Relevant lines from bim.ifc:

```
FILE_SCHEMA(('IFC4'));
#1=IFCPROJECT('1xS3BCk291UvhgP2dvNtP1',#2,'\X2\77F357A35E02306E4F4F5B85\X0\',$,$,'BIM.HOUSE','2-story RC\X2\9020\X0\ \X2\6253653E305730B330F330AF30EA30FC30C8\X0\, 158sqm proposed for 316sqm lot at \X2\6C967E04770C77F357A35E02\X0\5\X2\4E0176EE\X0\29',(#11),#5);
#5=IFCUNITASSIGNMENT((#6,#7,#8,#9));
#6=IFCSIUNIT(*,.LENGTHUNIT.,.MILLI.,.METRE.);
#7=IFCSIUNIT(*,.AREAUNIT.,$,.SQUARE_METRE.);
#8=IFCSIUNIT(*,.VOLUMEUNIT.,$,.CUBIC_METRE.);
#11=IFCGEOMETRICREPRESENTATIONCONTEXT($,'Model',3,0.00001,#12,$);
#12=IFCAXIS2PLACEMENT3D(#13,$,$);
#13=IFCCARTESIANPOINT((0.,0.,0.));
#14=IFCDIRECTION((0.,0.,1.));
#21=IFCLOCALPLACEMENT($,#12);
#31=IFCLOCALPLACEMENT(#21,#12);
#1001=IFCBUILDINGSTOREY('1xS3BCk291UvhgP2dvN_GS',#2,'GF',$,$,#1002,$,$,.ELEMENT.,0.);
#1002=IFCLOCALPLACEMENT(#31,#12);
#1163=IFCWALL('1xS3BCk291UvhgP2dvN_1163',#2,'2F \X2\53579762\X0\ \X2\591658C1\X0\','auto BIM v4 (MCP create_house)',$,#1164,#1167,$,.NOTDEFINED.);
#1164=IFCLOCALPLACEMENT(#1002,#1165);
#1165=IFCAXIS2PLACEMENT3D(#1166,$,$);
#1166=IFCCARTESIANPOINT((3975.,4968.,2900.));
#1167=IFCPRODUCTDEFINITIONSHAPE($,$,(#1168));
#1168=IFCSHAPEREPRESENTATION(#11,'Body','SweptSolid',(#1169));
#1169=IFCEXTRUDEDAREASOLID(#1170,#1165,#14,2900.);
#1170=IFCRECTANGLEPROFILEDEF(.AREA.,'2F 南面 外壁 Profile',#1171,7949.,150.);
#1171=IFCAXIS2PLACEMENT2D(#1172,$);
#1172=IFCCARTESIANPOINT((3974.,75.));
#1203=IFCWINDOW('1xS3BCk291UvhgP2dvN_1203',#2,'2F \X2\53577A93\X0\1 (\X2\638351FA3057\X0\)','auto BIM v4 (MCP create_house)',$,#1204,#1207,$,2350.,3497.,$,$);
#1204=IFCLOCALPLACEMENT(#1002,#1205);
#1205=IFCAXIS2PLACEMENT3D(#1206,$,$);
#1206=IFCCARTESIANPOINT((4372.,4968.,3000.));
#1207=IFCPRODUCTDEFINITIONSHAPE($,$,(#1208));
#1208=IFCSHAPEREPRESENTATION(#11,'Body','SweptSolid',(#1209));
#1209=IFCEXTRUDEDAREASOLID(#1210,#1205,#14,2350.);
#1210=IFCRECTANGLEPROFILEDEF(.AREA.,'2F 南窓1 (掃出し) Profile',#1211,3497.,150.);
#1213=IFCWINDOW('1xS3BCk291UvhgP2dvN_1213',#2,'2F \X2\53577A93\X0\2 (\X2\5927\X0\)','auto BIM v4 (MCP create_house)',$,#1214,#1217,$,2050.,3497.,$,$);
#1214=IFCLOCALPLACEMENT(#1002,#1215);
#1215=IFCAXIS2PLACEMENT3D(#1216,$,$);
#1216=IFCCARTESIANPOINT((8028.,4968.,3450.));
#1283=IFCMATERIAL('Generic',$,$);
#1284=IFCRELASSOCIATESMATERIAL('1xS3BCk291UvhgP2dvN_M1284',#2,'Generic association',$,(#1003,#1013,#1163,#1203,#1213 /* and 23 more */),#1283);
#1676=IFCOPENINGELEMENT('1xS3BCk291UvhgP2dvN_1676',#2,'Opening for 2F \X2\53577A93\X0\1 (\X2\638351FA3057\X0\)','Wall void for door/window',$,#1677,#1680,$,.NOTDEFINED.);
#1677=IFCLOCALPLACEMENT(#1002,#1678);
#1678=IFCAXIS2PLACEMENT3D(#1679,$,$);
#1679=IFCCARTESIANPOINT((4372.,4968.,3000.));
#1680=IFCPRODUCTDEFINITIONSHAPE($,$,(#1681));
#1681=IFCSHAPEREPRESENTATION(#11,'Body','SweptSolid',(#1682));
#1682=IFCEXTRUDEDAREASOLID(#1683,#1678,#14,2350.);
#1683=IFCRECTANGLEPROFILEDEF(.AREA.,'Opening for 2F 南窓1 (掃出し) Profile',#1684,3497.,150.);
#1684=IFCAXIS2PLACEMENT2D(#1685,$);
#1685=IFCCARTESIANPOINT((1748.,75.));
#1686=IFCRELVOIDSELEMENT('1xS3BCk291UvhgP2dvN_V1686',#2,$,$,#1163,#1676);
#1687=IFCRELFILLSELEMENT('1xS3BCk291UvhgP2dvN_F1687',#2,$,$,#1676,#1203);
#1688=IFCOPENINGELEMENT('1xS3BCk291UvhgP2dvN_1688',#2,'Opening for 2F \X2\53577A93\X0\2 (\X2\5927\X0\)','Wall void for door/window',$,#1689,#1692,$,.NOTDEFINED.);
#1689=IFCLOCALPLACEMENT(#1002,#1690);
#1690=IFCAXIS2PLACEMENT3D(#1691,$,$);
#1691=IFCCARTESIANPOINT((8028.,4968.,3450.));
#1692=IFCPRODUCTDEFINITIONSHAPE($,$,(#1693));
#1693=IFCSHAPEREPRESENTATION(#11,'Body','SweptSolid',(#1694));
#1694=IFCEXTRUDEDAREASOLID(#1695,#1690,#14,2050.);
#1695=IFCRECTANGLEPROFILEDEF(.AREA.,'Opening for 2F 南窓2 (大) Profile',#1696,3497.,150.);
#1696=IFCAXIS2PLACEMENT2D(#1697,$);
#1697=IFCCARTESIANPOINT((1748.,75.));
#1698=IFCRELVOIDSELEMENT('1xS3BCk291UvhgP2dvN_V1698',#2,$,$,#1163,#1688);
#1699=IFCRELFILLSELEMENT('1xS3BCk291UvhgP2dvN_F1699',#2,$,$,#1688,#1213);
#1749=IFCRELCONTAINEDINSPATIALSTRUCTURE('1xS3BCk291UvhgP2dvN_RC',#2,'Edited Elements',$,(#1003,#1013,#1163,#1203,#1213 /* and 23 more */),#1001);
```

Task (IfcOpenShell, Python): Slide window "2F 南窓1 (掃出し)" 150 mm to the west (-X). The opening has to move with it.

```python
import ifcopenshell
import ifcopenshell.api.geometry
import ifcopenshell.util.placement
import ifcopenshell.util.unit

model = ifcopenshell.open("bim.ifc")
unit_scale = ifcopenshell.util.unit.calculate_unit_scale(model)

window = model.by_guid("1xS3BCk291UvhgP2dvN_1203")
opening = window.FillsVoids[0].RelatingOpeningElement
wall = opening.VoidsElements[0].RelatingBuildingElement

wall_matrix = ifcopenshell.util.placement.get_local_placement(wall.ObjectPlacement)
shift = wall_matrix[:3, 0] * -0.15 / unit_scale
before = ifcopenshell.util.placement.get_local_placement(window.ObjectPlacement)[:3, 3].copy()

# The window is not placed relative to its opening, so move both.
for product in (opening, window):
    matrix = ifcopenshell.util.placement.get_local_placement(product.ObjectPlacement)
    matrix[:3, 3] += shift
    ifcopenshell.api.geometry.edit_object_placement(model, product=product, matrix=matrix, is_si=False)

after = ifcopenshell.util.placement.get_local_placement(window.ObjectPlacement)[:3, 3]
print("window moved by", (after - before).round(3) + 0.0)

model.write("bim_edited.ifc")
```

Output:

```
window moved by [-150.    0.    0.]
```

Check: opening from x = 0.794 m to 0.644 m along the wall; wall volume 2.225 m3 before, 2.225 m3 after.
